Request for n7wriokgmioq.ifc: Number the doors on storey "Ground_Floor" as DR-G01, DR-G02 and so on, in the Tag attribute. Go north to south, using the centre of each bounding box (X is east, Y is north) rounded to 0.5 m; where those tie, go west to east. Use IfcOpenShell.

First a look at what the model holds.

```python
import ifcopenshell
import ifcopenshell.util.element
import ifcopenshell.util.placement

model = ifcopenshell.open("n7wriokgmioq.ifc")
print(model.schema)
storey = next(s for s in model.by_type("IfcBuildingStorey") if s.Name == "Ground_Floor")
doors = [e for e in ifcopenshell.util.element.get_decomposition(storey) if e.is_a("IfcDoor")]
for e in sorted(doors, key=lambda e: e.id()):
    origin = ifcopenshell.util.placement.get_local_placement(e.ObjectPlacement)[:3, 3]
    print(e.id(), e.Tag, e.Name, origin.round(2) + 0.0, sep=" | ")
```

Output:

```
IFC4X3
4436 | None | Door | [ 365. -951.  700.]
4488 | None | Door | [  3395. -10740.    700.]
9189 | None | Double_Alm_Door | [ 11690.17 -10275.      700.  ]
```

```python
import ifcopenshell
import ifcopenshell.geom
import ifcopenshell.util.element
import ifcopenshell.util.shape

model = ifcopenshell.open("n7wriokgmioq.ifc")
settings = ifcopenshell.geom.settings()
settings.set("use-world-coords", True)


def centre(element):
    shape = ifcopenshell.geom.create_shape(settings, element)
    return ifcopenshell.util.shape.get_bbox_centroid(shape.geometry)


storey = next(s for s in model.by_type("IfcBuildingStorey") if s.Name == "Ground_Floor")
doors = [e for e in ifcopenshell.util.element.get_decomposition(storey) if e.is_a("IfcDoor")]

# Insertion points can sit at a corner or the storey origin, so sort by the geometry (in metres).
centres = {e: centre(e) for e in doors}
doors.sort(key=lambda e: (-round(centres[e][1] / 0.5), centres[e][0]))

for i, e in enumerate(doors, start=1):
    number = f"DR-G{i:02d}"
    e.Tag = number
    print(e.id(), number)

model.write("n7wriokgmioq_edited.ifc")
```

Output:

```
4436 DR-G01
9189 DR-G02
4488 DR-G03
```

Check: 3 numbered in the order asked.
